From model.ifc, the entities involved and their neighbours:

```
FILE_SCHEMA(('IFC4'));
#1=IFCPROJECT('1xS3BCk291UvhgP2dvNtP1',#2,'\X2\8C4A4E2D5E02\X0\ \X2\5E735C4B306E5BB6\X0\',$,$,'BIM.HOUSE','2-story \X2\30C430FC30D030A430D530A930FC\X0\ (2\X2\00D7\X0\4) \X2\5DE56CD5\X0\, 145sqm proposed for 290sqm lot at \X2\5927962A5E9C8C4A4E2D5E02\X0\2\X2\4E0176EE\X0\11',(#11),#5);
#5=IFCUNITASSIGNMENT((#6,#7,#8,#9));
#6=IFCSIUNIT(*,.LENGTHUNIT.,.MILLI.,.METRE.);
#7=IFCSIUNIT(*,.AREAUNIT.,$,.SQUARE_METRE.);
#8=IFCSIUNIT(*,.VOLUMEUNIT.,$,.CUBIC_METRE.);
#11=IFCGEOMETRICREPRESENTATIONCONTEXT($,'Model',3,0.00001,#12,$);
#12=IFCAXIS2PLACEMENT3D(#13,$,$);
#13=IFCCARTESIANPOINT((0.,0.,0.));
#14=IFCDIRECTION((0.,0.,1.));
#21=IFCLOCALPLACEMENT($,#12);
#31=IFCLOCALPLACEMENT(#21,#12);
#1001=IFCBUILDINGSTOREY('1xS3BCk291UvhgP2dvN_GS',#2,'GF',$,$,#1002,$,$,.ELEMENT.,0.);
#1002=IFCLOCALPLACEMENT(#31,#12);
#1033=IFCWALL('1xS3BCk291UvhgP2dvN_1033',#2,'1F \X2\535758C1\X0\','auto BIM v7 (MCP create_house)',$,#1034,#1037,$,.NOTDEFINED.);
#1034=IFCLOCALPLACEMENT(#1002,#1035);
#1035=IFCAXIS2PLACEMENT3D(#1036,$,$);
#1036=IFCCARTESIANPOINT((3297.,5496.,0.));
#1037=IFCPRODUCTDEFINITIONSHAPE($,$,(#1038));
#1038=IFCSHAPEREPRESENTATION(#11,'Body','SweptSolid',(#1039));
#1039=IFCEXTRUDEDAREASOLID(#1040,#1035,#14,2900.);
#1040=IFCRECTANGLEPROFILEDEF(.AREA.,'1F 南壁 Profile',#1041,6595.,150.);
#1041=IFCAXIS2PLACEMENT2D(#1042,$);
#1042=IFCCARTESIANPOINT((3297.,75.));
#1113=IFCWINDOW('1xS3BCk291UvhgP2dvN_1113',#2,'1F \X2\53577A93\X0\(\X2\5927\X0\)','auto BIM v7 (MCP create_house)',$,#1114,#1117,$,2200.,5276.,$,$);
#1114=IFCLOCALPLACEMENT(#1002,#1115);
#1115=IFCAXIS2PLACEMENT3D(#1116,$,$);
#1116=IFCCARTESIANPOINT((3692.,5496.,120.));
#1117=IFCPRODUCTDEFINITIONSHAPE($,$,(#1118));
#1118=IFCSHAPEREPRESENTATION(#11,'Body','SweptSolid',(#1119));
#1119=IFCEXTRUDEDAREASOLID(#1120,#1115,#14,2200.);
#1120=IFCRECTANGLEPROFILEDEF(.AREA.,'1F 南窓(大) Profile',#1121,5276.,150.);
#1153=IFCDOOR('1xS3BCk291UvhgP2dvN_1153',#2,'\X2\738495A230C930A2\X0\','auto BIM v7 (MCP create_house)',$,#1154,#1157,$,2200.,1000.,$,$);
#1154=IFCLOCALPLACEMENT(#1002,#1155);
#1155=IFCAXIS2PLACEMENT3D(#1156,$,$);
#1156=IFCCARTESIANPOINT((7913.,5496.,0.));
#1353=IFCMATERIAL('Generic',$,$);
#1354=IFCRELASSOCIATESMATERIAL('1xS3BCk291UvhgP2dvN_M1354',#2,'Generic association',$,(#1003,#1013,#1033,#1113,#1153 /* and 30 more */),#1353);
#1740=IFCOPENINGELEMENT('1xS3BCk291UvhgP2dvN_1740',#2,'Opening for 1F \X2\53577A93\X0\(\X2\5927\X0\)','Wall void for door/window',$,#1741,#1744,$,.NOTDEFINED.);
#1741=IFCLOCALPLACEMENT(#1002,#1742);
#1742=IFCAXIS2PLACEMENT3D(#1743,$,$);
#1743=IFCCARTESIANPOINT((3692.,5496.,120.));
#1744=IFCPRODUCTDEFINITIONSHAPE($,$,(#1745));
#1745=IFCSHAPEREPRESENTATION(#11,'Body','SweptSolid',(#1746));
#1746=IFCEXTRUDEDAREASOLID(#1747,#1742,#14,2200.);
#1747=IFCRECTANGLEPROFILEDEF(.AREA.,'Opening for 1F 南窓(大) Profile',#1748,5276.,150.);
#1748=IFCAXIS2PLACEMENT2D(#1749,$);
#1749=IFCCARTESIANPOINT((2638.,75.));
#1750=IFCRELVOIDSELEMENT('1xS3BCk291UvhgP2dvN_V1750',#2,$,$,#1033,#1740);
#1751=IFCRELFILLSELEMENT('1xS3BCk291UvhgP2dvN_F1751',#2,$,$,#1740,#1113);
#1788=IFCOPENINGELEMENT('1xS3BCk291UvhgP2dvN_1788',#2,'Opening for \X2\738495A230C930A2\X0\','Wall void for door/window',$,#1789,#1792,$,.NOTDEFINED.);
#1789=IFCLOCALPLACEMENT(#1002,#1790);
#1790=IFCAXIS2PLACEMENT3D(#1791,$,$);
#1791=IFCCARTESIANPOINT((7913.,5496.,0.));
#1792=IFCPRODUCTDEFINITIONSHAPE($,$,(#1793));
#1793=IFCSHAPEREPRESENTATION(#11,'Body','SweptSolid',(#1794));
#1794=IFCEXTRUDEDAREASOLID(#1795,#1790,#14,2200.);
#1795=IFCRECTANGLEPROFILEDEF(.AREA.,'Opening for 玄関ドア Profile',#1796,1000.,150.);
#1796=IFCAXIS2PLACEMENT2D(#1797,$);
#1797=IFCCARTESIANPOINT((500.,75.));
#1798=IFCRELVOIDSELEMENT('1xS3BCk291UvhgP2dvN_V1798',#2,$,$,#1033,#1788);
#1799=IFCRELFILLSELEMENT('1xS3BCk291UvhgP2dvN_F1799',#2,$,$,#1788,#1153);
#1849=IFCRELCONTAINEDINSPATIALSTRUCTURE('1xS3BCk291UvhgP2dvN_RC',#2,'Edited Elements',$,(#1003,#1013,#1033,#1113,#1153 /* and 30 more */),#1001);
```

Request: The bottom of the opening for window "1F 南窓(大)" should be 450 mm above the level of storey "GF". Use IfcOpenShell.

```python
import numpy as np
import ifcopenshell
import ifcopenshell.api.geometry
import ifcopenshell.geom
import ifcopenshell.util.element
import ifcopenshell.util.placement
import ifcopenshell.util.shape
import ifcopenshell.util.unit

model = ifcopenshell.open("model.ifc")
unit_scale = ifcopenshell.util.unit.calculate_unit_scale(model)

window = model.by_id(1113)
opening = window.FillsVoids[0].RelatingOpeningElement
storey = ifcopenshell.util.element.get_container(window, ifc_class="IfcBuildingStorey")
level = ifcopenshell.util.placement.get_local_placement(storey.ObjectPlacement)[2, 3]

# The opening's origin need not be at the sill, so measure its lowest point.
shape = ifcopenshell.geom.create_shape(ifcopenshell.geom.settings(), opening)
bottom = ifcopenshell.util.shape.get_shape_bottom_elevation(shape, shape.geometry) / unit_scale
dz = level + 450.0 - bottom

shift = np.array([0.0, 0.0, dz])
# The window is not placed relative to its opening, so move both.
for product in (opening, window):
    matrix = ifcopenshell.util.placement.get_local_placement(product.ObjectPlacement)
    matrix[:3, 3] += shift
    ifcopenshell.api.geometry.edit_object_placement(model, product=product, matrix=matrix, is_si=False)

print(f"moved by {dz * unit_scale:+.3f} m")

model.write("model_edited.ifc")
```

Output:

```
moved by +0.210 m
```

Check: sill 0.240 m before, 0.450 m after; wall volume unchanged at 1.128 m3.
